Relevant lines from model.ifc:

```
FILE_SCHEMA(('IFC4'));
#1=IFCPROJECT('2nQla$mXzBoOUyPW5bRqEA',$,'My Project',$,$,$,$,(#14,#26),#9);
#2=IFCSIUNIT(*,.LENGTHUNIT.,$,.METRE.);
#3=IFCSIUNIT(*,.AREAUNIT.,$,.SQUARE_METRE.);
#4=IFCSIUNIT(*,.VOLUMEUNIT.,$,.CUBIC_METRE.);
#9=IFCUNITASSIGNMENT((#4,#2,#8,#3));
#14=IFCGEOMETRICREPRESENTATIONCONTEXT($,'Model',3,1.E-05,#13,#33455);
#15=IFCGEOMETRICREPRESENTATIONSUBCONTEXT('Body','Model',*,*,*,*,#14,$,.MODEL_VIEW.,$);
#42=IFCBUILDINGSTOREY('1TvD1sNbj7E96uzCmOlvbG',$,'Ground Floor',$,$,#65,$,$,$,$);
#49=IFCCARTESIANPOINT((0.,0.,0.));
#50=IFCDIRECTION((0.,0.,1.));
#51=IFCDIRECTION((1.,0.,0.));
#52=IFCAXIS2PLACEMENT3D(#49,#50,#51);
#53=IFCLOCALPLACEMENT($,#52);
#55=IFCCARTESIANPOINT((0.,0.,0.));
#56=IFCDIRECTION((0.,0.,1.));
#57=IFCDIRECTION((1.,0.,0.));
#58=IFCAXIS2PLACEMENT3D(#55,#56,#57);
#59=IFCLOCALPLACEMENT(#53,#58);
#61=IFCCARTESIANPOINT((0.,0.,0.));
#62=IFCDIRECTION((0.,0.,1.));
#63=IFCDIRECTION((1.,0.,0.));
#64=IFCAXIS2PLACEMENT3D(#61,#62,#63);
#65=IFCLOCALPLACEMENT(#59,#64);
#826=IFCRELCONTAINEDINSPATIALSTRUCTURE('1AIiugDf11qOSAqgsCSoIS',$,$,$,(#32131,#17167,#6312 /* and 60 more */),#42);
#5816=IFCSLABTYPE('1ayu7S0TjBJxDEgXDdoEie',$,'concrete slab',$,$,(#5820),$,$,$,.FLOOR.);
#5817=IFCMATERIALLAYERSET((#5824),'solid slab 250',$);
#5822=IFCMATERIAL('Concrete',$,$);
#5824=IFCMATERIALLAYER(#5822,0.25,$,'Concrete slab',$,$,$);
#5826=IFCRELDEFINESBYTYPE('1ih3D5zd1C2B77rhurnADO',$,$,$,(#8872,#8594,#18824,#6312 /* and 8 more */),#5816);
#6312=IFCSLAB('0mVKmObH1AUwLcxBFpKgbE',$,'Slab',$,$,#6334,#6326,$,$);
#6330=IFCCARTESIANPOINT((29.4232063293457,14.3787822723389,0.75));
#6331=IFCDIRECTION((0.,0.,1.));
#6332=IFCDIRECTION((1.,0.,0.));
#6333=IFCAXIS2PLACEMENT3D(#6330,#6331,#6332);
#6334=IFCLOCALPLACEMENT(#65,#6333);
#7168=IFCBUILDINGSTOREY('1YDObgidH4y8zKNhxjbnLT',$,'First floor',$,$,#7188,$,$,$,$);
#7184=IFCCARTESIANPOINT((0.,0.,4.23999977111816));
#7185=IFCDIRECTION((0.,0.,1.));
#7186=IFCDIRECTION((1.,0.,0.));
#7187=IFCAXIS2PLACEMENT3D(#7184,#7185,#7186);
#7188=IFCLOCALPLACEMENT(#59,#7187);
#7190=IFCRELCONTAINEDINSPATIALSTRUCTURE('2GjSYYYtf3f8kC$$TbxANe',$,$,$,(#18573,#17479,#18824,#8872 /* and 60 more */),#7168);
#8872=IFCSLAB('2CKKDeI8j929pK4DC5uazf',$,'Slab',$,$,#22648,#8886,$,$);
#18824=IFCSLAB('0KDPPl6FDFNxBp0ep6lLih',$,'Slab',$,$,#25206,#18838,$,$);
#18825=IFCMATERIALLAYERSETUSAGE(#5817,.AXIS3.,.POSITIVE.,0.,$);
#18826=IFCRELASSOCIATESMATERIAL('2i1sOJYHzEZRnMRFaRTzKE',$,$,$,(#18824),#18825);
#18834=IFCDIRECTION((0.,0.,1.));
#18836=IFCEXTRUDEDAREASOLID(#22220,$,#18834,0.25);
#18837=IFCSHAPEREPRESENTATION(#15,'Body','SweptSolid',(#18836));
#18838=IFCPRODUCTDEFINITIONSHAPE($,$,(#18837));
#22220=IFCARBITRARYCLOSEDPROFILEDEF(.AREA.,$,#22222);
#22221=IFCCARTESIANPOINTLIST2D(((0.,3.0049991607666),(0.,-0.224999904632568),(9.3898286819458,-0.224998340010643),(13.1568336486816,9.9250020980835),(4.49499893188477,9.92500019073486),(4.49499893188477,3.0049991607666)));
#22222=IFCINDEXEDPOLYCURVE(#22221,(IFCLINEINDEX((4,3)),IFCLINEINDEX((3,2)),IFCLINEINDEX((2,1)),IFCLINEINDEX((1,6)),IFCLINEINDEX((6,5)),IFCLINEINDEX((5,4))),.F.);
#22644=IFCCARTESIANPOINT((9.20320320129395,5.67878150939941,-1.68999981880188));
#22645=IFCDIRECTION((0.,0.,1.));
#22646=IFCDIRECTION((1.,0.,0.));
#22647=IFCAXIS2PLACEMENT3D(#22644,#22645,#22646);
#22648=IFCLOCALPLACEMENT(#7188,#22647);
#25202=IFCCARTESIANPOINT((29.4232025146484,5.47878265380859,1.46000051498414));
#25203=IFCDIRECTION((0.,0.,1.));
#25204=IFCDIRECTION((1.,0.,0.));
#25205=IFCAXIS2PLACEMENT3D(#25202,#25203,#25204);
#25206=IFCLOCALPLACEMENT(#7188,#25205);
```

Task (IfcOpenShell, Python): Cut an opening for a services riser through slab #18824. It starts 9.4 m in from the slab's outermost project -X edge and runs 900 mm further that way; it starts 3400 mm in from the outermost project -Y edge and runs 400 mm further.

```python
import numpy as np
import ifcopenshell
import ifcopenshell.api.feature
import ifcopenshell.api.geometry
import ifcopenshell.api.root
import ifcopenshell.geom
import ifcopenshell.util.placement
import ifcopenshell.util.representation
import ifcopenshell.util.shape
import ifcopenshell.util.unit

model = ifcopenshell.open("model.ifc")
unit_scale = ifcopenshell.util.unit.calculate_unit_scale(model)
settings = ifcopenshell.geom.settings()


def volume(element):
    """Net volume in cubic metres, openings subtracted."""
    shape = ifcopenshell.geom.create_shape(settings, element)
    return ifcopenshell.util.shape.get_volume(shape.geometry)


slab = model.by_id(18824)
before = volume(slab)

# Extent in the slab's own axes, in metres. The edges named are its -X and -Y sides.
slab_shape = ifcopenshell.geom.create_shape(settings, slab)
vertices = ifcopenshell.util.shape.get_vertices(slab_shape.geometry)
x_min, y_min, bottom = vertices.min(axis=0)
top = vertices[:, 2].max()

opening = ifcopenshell.api.root.create_entity(model, ifc_class="IfcOpeningElement", name="Services riser opening", predefined_type="OPENING")
context = ifcopenshell.util.representation.get_context(model, "Model", "Body", "MODEL_VIEW")
width, depth = 0.9, 0.4
outline = [(0.0, 0.0), (width, 0.0), (width, depth), (0.0, depth), (0.0, 0.0)]
# Overshoot both faces by 50 mm so the cut is clean.
shape = ifcopenshell.api.geometry.add_slab_representation(
    model, context=context, depth=top - bottom + 0.1, polyline=outline
)
ifcopenshell.api.geometry.assign_representation(model, product=opening, representation=shape)

matrix = ifcopenshell.util.placement.get_local_placement(slab.ObjectPlacement)
matrix[:, 3] = matrix @ np.append(np.array([x_min + 9.4, y_min + 3.4, bottom - 0.05]) / unit_scale, 1.0)
ifcopenshell.api.geometry.edit_object_placement(model, product=opening, matrix=matrix, is_si=False)
ifcopenshell.api.feature.add_feature(model, feature=opening, element=slab)

after = volume(slab)

print(f"slab volume {before:.3f} -> {after:.3f} m3")

model.write("model_rev.ifc")
```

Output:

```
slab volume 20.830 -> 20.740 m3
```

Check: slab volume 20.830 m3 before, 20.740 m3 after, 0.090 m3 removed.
